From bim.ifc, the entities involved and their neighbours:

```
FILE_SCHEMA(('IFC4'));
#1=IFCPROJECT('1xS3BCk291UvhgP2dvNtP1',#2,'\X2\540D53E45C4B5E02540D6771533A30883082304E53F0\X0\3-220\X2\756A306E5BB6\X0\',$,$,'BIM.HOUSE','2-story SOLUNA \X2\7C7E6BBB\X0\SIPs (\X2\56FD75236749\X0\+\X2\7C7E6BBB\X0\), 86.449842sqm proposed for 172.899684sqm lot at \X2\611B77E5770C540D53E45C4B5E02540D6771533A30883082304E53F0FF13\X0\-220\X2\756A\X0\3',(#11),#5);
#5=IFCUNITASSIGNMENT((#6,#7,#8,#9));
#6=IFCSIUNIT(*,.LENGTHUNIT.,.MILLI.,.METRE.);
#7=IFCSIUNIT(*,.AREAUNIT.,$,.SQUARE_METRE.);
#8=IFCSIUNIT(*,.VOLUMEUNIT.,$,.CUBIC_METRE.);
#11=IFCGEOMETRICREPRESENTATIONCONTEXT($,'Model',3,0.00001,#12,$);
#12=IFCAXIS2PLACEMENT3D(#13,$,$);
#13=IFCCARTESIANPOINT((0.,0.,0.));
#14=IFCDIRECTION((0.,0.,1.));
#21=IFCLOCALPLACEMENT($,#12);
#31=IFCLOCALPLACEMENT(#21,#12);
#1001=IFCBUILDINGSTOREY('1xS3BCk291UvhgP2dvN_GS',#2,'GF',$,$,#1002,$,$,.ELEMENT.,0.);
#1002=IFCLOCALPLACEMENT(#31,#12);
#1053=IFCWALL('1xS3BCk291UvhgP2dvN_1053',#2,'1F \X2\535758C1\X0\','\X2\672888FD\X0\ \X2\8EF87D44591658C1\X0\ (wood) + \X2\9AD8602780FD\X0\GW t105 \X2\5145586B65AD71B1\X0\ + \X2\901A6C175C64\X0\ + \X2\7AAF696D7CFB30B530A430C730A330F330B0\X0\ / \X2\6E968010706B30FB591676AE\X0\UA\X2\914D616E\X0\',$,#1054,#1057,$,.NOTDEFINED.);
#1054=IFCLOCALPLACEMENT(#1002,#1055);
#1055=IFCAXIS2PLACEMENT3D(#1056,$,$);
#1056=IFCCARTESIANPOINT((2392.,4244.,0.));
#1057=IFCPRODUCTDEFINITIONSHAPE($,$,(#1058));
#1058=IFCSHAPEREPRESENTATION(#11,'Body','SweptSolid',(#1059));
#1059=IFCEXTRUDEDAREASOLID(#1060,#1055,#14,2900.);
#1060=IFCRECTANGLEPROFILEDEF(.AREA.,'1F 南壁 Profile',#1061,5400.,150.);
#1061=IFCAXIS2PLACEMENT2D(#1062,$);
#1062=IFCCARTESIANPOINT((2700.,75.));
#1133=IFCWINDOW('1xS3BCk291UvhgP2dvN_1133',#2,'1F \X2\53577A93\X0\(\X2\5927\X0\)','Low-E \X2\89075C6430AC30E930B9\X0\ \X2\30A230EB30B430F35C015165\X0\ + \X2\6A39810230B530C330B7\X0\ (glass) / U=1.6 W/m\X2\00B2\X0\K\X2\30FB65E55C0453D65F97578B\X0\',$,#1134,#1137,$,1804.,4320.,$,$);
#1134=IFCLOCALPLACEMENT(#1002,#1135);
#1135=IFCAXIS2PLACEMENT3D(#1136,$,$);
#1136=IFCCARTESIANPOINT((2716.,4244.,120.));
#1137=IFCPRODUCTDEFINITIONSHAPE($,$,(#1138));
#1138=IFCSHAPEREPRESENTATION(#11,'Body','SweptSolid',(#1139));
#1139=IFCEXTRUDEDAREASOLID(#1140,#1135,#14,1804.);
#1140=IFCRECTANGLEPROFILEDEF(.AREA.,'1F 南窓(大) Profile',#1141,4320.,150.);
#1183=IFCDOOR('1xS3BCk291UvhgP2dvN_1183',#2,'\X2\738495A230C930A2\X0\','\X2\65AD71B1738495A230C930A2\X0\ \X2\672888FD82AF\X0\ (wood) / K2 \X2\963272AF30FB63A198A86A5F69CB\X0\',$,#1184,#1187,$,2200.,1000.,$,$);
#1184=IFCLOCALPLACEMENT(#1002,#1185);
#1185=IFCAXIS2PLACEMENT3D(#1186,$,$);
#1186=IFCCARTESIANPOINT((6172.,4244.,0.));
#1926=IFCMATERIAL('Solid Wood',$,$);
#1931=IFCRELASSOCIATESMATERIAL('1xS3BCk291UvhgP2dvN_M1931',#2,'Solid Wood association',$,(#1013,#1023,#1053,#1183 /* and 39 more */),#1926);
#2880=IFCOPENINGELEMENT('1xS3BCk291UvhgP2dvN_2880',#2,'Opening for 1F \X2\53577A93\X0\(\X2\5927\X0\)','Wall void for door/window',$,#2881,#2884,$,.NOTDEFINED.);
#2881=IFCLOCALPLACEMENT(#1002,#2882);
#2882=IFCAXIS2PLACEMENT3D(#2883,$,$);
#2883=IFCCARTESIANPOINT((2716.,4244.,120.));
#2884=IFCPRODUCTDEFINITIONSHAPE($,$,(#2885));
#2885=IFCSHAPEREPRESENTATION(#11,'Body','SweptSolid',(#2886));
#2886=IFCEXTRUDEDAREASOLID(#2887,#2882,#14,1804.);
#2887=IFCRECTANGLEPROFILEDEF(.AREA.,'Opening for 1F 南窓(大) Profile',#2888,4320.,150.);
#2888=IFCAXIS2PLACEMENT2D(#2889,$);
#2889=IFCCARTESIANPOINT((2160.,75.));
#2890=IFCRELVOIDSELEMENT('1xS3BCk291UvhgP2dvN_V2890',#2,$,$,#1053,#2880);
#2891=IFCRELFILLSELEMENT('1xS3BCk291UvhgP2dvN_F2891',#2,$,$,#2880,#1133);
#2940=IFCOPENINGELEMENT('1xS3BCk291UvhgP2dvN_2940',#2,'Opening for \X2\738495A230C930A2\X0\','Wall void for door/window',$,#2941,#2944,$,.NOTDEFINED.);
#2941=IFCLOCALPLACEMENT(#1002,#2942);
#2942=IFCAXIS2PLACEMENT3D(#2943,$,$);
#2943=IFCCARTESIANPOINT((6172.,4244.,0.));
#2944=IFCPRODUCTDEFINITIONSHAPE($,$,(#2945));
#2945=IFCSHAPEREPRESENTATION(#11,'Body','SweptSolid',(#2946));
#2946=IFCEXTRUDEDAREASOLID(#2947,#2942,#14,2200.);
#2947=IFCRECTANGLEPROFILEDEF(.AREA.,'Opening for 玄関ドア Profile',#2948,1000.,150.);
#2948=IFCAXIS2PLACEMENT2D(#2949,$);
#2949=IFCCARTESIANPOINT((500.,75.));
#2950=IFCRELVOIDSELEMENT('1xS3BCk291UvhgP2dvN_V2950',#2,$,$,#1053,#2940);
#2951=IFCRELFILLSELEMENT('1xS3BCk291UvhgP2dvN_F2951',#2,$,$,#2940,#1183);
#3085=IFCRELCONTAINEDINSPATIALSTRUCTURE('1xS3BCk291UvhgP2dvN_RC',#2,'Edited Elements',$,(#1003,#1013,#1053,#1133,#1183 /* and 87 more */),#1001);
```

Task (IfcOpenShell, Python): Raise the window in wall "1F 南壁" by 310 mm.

```python
import numpy as np
import ifcopenshell
import ifcopenshell.api.geometry
import ifcopenshell.util.placement
import ifcopenshell.util.unit

model = ifcopenshell.open("bim.ifc")
unit_scale = ifcopenshell.util.unit.calculate_unit_scale(model)

window = model.by_guid("1xS3BCk291UvhgP2dvN_1133")
opening = window.FillsVoids[0].RelatingOpeningElement
dz = 0.31 / unit_scale

shift = np.array([0.0, 0.0, dz])
# The window is not placed relative to its opening, so move both.
for product in (opening, window):
    matrix = ifcopenshell.util.placement.get_local_placement(product.ObjectPlacement)
    matrix[:3, 3] += shift
    ifcopenshell.api.geometry.edit_object_placement(model, product=product, matrix=matrix, is_si=False)

print(f"moved by {dz * unit_scale:+.3f} m")

model.write("bim-out.ifc")
```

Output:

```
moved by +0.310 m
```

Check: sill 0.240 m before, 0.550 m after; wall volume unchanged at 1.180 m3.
